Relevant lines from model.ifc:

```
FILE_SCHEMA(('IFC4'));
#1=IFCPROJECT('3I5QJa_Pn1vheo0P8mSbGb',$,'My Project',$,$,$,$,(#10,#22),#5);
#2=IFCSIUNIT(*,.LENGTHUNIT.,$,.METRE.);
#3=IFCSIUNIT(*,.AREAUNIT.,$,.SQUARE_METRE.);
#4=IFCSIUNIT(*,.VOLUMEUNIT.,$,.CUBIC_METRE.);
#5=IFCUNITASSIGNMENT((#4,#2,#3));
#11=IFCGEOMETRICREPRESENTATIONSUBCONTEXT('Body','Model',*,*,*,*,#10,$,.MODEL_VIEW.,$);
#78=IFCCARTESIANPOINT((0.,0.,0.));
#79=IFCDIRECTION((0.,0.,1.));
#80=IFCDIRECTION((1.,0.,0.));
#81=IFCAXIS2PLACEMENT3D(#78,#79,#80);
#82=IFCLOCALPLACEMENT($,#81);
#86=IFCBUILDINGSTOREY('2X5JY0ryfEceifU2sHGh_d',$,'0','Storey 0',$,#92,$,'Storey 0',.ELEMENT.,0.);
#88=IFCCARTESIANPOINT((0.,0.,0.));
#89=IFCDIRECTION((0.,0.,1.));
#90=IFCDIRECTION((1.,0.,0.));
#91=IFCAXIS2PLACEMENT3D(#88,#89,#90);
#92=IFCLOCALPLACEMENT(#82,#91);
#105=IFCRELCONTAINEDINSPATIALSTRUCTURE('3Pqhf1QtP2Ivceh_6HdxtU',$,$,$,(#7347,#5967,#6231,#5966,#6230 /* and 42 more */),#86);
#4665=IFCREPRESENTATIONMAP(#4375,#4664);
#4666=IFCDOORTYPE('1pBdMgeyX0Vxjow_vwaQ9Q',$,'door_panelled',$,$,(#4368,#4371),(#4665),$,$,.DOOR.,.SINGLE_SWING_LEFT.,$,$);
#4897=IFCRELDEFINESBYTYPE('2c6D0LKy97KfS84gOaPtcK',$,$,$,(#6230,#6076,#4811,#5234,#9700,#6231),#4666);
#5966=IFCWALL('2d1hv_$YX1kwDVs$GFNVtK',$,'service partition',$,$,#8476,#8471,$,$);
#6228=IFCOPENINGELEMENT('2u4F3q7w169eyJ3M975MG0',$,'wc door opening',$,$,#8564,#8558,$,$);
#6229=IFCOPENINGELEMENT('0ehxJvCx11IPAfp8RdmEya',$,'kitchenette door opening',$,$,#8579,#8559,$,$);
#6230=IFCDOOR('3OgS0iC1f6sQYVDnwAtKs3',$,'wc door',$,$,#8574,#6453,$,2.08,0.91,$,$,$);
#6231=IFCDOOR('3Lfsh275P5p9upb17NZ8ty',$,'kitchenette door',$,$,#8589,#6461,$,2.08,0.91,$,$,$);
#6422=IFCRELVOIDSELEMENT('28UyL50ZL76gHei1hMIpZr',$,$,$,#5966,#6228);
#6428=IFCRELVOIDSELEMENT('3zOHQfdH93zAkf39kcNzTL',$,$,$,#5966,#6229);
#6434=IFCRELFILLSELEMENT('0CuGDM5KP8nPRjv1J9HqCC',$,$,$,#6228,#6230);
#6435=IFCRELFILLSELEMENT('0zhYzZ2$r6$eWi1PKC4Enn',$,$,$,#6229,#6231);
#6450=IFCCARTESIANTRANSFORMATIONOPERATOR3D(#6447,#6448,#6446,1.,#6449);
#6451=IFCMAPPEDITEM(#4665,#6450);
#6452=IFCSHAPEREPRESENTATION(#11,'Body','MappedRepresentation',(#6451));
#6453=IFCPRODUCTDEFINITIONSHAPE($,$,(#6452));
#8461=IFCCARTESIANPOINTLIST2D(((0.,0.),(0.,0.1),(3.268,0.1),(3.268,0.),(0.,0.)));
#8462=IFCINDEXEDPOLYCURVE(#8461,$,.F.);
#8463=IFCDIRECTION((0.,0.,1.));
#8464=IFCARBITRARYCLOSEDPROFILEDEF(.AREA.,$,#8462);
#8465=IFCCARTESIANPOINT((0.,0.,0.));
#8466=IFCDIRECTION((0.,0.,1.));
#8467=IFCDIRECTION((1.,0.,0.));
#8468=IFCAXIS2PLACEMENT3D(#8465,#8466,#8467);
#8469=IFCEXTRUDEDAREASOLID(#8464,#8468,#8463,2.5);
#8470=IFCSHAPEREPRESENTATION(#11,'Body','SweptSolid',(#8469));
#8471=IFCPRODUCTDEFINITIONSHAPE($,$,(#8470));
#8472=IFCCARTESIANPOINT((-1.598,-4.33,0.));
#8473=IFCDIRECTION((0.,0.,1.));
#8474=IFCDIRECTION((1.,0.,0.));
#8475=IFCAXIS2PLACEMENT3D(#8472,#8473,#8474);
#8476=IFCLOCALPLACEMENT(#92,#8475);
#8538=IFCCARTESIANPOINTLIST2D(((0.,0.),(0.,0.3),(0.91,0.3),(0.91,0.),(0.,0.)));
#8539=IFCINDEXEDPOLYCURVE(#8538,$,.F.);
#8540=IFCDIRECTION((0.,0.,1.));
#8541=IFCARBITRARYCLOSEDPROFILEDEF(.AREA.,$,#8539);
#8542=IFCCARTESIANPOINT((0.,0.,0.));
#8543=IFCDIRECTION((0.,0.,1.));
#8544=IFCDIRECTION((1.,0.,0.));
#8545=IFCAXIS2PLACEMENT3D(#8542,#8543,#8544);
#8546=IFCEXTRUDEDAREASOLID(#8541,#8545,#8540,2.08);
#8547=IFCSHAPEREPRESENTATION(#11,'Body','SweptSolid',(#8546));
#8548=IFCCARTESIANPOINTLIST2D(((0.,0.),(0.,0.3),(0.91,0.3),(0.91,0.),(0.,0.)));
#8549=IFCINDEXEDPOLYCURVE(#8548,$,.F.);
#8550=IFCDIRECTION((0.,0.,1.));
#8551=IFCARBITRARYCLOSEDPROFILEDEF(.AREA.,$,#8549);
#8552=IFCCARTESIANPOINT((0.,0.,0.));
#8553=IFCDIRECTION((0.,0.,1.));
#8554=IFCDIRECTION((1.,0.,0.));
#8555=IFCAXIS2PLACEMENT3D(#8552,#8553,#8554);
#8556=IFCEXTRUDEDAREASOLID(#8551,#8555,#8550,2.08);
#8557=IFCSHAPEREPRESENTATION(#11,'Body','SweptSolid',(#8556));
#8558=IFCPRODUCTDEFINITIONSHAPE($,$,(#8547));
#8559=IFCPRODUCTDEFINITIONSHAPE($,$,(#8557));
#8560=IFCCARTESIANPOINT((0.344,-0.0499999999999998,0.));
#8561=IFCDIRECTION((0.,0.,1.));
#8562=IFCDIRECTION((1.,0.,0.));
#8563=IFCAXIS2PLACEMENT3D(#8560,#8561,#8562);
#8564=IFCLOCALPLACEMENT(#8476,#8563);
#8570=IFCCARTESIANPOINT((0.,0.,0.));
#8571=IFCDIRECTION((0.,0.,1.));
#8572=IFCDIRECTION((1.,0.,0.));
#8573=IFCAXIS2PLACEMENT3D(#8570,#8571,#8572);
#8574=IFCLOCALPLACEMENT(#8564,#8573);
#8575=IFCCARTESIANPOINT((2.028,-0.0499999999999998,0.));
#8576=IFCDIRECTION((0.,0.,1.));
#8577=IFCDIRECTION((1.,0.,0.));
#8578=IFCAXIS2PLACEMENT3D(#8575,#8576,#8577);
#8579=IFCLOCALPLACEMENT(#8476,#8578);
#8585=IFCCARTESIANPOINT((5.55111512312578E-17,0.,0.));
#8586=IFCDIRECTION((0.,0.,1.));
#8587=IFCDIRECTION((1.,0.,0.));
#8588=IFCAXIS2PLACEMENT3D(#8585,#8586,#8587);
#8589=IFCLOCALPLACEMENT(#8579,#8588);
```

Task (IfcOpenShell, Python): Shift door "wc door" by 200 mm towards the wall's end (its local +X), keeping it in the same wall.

```python
import ifcopenshell
import ifcopenshell.api.geometry
import ifcopenshell.util.placement
import ifcopenshell.util.unit

model = ifcopenshell.open("model.ifc")
unit_scale = ifcopenshell.util.unit.calculate_unit_scale(model)

door = model.by_guid("3OgS0iC1f6sQYVDnwAtKs3")
opening = door.FillsVoids[0].RelatingOpeningElement
wall = opening.VoidsElements[0].RelatingBuildingElement

wall_matrix = ifcopenshell.util.placement.get_local_placement(wall.ObjectPlacement)
shift = wall_matrix[:3, 0] * 0.2 / unit_scale
before = ifcopenshell.util.placement.get_local_placement(door.ObjectPlacement)[:3, 3].copy()

# The door is placed relative to its opening, so it follows when the opening moves.
matrix = ifcopenshell.util.placement.get_local_placement(opening.ObjectPlacement)
matrix[:3, 3] += shift
ifcopenshell.api.geometry.edit_object_placement(
    model, product=opening, matrix=matrix, is_si=False, should_transform_children=True
)

after = ifcopenshell.util.placement.get_local_placement(door.ObjectPlacement)[:3, 3]
print("door moved by", (after - before).round(3) + 0.0)

model.write("model_v2.ifc")
```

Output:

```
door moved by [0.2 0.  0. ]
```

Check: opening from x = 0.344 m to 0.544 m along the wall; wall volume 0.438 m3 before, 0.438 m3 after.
